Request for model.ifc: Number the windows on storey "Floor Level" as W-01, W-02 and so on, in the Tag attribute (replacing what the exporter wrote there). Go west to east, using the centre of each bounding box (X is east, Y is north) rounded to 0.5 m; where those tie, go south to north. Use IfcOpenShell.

First a look at what the model holds.

```python
import ifcopenshell
import ifcopenshell.util.element
import ifcopenshell.util.placement

model = ifcopenshell.open("model.ifc")
print(model.schema)
storey = next(s for s in model.by_type("IfcBuildingStorey") if s.Name == "Floor Level")
windows = [e for e in ifcopenshell.util.element.get_decomposition(storey) if e.is_a("IfcWindow")]
for e in sorted(windows, key=lambda e: e.id()):
    origin = ifcopenshell.util.placement.get_local_placement(e.ObjectPlacement)[:3, 3]
    print(e.id(), e.Tag, e.Name, origin.round(2) + 0.0, sep=" | ")
```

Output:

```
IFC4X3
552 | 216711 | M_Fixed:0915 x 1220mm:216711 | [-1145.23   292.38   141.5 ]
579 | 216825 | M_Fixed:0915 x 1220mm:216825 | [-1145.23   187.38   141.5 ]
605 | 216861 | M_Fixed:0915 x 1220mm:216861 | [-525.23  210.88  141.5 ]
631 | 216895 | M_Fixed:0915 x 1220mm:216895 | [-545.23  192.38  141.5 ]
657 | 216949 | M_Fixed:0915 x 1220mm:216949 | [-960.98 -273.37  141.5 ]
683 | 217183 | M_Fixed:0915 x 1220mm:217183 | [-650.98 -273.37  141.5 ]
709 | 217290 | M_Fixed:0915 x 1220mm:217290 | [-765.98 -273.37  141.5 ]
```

```python
import ifcopenshell
import ifcopenshell.geom
import ifcopenshell.util.element
import ifcopenshell.util.shape

model = ifcopenshell.open("model.ifc")
settings = ifcopenshell.geom.settings()
settings.set("use-world-coords", True)


def centre(element):
    shape = ifcopenshell.geom.create_shape(settings, element)
    return ifcopenshell.util.shape.get_bbox_centroid(shape.geometry)


storey = next(s for s in model.by_type("IfcBuildingStorey") if s.Name == "Floor Level")
windows = [e for e in ifcopenshell.util.element.get_decomposition(storey) if e.is_a("IfcWindow")]

# Insertion points can sit at a corner or the storey origin, so sort by the geometry (in metres).
centres = {e: centre(e) for e in windows}
windows.sort(key=lambda e: (round(centres[e][0] / 0.5), centres[e][1]))

for i, e in enumerate(windows, start=1):
    number = f"W-{i:02d}"
    e.Tag = number
    print(e.id(), number)

model.write("model_rev.ifc")
```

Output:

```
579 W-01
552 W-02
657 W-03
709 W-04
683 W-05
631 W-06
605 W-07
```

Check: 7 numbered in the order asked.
